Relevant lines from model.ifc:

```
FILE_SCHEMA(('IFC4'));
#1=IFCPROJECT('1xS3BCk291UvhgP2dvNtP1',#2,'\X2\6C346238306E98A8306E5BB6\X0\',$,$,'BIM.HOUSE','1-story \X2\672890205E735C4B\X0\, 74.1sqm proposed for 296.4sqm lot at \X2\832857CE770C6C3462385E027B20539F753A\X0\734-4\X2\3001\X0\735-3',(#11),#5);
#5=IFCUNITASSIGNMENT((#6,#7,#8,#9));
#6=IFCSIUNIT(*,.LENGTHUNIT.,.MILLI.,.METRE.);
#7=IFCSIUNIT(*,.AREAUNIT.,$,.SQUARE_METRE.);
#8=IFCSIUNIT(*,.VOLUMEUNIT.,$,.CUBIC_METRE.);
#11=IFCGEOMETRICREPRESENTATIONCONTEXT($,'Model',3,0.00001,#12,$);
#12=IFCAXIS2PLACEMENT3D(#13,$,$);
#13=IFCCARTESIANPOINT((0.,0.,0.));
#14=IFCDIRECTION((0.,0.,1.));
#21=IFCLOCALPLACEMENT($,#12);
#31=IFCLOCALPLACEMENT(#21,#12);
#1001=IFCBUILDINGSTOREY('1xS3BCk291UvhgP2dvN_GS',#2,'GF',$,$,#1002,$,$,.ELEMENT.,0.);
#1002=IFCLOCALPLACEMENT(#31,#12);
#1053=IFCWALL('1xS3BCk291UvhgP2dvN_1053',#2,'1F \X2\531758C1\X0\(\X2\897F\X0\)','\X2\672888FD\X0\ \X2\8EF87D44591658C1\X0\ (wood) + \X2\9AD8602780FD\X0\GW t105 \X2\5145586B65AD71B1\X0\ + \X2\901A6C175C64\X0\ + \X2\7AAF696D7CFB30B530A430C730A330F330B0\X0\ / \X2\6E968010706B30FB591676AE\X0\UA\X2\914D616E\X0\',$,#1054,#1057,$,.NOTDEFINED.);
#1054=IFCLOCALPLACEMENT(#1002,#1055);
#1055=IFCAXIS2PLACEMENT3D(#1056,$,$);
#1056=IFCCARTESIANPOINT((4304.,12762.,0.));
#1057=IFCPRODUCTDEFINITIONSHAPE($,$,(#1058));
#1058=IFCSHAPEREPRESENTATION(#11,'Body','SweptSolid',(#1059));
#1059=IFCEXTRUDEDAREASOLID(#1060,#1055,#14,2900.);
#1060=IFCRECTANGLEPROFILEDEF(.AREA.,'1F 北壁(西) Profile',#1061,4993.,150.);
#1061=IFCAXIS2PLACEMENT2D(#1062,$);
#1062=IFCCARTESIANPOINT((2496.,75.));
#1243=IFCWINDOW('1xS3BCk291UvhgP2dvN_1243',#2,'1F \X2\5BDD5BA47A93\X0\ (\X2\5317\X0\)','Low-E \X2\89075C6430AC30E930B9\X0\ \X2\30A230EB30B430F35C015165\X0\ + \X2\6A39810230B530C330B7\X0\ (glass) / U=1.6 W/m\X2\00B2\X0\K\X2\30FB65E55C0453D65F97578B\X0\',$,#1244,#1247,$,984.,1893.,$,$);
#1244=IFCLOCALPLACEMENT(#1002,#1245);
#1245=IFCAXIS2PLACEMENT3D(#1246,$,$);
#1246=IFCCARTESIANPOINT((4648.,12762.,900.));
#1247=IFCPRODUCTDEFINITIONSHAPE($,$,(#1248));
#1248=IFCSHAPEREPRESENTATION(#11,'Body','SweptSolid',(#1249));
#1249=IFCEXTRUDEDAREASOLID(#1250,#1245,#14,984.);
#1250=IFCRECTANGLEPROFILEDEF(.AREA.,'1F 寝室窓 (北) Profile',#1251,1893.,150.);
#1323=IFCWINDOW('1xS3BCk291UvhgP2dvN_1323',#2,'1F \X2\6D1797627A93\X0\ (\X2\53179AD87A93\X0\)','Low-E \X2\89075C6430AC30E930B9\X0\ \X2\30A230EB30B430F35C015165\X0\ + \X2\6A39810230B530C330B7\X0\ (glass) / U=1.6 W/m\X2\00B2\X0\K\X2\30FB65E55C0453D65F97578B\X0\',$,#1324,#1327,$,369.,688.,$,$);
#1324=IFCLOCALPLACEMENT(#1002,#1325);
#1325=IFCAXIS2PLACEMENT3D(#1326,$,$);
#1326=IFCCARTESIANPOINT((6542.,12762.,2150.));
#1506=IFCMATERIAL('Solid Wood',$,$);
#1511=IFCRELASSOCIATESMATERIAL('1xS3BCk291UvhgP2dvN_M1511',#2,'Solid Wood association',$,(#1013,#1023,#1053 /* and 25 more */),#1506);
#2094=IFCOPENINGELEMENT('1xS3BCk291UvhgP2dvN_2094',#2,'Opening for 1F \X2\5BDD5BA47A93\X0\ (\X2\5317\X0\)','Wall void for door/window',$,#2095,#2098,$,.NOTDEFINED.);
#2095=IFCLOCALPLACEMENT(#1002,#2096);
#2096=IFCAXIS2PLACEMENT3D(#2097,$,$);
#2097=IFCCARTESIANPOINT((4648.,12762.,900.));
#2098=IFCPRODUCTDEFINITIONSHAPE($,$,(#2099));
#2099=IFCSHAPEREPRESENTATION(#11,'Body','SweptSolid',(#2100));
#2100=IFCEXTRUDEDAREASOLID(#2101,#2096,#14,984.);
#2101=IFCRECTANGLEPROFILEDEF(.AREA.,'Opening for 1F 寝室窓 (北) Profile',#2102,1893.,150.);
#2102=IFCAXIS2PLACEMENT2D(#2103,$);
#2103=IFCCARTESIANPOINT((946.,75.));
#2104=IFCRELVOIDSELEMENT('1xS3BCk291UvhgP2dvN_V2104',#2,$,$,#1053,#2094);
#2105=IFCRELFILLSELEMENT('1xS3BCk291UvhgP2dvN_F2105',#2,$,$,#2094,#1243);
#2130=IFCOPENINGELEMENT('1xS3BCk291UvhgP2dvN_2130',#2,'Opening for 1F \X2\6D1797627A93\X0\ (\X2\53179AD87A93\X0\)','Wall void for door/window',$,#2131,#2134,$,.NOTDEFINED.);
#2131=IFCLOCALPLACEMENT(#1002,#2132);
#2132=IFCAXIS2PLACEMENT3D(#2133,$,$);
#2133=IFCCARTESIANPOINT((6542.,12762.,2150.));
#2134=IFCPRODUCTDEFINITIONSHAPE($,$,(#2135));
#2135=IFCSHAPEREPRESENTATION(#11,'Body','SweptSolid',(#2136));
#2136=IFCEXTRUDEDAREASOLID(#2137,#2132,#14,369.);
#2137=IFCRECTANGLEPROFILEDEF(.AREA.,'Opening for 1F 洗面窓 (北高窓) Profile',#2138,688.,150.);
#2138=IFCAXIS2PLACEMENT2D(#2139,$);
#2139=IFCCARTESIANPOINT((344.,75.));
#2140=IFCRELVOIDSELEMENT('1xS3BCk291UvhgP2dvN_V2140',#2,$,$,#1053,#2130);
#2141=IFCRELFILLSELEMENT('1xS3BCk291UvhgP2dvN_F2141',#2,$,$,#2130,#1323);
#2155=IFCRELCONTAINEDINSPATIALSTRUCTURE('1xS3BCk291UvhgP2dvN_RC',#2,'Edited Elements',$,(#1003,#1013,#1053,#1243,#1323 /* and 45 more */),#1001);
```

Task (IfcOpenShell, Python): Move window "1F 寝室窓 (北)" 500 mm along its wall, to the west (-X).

```python
import ifcopenshell
import ifcopenshell.api.geometry
import ifcopenshell.util.placement

model = ifcopenshell.open("model.ifc")

window = model.by_guid("1xS3BCk291UvhgP2dvN_1243")
opening = window.FillsVoids[0].RelatingOpeningElement
wall = opening.VoidsElements[0].RelatingBuildingElement

wall_matrix = ifcopenshell.util.placement.get_local_placement(wall.ObjectPlacement)
shift = wall_matrix[:3, 0] * -500.0
before = ifcopenshell.util.placement.get_local_placement(window.ObjectPlacement)[:3, 3].copy()

# The window is not placed relative to its opening, so move both.
for product in (opening, window):
    matrix = ifcopenshell.util.placement.get_local_placement(product.ObjectPlacement)
    matrix[:3, 3] += shift
    ifcopenshell.api.geometry.edit_object_placement(model, product=product, matrix=matrix, is_si=False)

after = ifcopenshell.util.placement.get_local_placement(window.ObjectPlacement)[:3, 3]
print("window moved by", (after - before).round(3) + 0.0)

model.write("model_edited.ifc")
```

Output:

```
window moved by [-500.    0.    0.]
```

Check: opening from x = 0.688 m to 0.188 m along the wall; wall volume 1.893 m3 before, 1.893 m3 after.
